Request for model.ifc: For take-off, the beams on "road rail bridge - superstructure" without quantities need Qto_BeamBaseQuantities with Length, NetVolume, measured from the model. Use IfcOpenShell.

First a look at what the model holds.

```python
import ifcopenshell
import ifcopenshell.util.element
import ifcopenshell.util.unit

model = ifcopenshell.open("model.ifc")
print(model.schema)
for unit_type in ("LENGTHUNIT", "AREAUNIT", "VOLUMEUNIT"):
    print(unit_type, ifcopenshell.util.unit.calculate_unit_scale(model, unit_type))
storey = next(s for s in model.by_type("IfcBuildingStorey") if s.Name == "road rail bridge - superstructure")
beams = [e for e in ifcopenshell.util.element.get_decomposition(storey) if e.is_a("IfcBeam")]
for e in sorted(beams, key=lambda e: e.id()):
    print(e.id(), e.is_a(), e.Name, list(ifcopenshell.util.element.get_psets(e, qtos_only=True)), sep=" | ")
```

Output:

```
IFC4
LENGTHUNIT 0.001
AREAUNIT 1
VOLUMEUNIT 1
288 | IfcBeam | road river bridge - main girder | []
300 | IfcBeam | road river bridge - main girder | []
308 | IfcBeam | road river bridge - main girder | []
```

```python
import ifcopenshell
import ifcopenshell.api.pset
import ifcopenshell.geom
import ifcopenshell.util.element
import ifcopenshell.util.shape
import ifcopenshell.util.unit

model = ifcopenshell.open("model.ifc")
unit_scale = ifcopenshell.util.unit.calculate_unit_scale(model)
volume_scale = ifcopenshell.util.unit.calculate_unit_scale(model, "VOLUMEUNIT")
settings = ifcopenshell.geom.settings()

storey = next(s for s in model.by_type("IfcBuildingStorey") if s.Name == "road rail bridge - superstructure")
beams = [e for e in ifcopenshell.util.element.get_decomposition(storey) if e.is_a("IfcBeam")]

for e in sorted(beams, key=lambda e: e.id()):
    if ifcopenshell.util.element.get_psets(e, qtos_only=True, should_inherit=False):
        continue
    # Geometry comes back in metres, in the element's own axes.
    shape = ifcopenshell.geom.create_shape(settings, e)
    values = {
        "Length": ifcopenshell.util.shape.get_max_xyz(shape.geometry) / unit_scale,
        "NetVolume": ifcopenshell.util.shape.get_volume(shape.geometry) / volume_scale,
    }
    qto = ifcopenshell.api.pset.add_qto(model, product=e, name="Qto_BeamBaseQuantities")
    ifcopenshell.api.pset.edit_qto(model, qto=qto, properties=values)
    print(e.id(), {k: round(v, 3) for k, v in values.items()})

model.write("model_updated.ifc")
```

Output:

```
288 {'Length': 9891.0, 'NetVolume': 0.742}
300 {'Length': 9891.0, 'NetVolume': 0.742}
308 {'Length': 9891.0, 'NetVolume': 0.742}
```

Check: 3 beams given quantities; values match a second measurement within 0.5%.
